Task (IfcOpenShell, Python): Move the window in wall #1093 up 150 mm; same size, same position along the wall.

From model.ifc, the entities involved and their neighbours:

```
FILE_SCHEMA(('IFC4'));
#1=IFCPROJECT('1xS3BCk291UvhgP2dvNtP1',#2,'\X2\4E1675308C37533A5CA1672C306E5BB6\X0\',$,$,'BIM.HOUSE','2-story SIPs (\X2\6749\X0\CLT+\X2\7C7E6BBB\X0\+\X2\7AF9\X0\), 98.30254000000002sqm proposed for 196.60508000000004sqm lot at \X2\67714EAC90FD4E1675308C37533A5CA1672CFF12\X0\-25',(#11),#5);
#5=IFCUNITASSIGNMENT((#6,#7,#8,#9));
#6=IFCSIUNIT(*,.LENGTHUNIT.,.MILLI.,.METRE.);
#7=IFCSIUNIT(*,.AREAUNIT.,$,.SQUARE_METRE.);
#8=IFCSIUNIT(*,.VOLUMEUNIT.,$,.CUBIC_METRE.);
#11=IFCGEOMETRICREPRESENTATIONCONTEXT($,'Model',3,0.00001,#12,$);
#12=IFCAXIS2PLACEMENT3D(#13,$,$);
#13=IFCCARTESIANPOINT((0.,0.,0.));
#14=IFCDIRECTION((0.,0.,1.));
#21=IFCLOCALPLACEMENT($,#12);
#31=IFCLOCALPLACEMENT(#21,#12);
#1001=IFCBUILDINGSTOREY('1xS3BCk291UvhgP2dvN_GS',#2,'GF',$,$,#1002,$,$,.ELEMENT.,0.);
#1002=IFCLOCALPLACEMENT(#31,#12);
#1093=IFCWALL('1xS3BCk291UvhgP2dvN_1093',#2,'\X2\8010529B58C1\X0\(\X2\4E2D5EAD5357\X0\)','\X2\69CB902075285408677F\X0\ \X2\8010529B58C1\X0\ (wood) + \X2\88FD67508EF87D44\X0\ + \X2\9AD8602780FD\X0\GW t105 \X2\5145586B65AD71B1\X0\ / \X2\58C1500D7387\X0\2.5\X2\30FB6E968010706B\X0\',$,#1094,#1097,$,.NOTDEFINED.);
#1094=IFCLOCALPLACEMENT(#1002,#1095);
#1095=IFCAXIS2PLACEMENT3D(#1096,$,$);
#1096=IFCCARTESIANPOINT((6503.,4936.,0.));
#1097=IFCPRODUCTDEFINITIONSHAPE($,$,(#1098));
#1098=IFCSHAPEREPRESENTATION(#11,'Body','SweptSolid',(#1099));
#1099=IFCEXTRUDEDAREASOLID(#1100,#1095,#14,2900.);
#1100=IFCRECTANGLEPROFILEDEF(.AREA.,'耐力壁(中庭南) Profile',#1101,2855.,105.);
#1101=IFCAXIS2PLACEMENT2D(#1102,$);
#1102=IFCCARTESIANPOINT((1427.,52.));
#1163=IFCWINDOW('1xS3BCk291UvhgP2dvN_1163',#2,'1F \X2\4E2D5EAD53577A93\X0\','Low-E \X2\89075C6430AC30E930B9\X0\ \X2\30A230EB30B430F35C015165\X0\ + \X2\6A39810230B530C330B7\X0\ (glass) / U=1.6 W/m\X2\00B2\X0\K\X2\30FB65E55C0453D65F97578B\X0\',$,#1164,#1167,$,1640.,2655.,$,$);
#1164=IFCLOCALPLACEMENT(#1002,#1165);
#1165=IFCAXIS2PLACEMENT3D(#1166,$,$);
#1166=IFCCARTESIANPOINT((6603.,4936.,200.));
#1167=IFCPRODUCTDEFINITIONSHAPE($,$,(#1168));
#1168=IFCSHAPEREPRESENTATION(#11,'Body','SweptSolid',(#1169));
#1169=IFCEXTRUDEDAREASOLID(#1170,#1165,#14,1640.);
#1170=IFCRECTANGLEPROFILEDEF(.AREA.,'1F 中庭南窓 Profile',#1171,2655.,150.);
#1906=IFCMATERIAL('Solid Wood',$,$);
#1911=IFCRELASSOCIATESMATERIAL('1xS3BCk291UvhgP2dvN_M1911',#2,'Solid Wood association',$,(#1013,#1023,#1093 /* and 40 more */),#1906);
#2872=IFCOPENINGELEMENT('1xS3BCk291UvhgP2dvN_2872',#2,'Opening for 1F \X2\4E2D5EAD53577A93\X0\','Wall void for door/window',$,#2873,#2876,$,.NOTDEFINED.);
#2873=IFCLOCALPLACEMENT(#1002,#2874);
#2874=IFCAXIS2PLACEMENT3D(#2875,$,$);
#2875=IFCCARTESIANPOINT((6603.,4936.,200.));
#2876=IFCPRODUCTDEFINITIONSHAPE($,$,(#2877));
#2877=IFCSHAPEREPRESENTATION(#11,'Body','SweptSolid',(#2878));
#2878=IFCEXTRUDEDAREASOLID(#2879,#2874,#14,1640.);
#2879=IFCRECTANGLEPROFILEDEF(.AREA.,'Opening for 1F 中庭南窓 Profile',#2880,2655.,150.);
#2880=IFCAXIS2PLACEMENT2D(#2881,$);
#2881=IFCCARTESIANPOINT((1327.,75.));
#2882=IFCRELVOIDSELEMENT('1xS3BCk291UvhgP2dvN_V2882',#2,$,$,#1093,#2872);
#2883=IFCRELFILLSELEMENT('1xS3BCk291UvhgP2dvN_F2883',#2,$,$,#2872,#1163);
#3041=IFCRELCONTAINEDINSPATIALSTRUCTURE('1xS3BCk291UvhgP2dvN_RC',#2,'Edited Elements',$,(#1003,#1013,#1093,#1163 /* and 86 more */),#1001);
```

```python
import numpy as np
import ifcopenshell
import ifcopenshell.api.geometry
import ifcopenshell.util.placement
import ifcopenshell.util.unit

model = ifcopenshell.open("model.ifc")
unit_scale = ifcopenshell.util.unit.calculate_unit_scale(model)

window = model.by_id(1163)
opening = window.FillsVoids[0].RelatingOpeningElement
dz = 150.0

shift = np.array([0.0, 0.0, dz])
# The window is not placed relative to its opening, so move both.
for product in (opening, window):
    matrix = ifcopenshell.util.placement.get_local_placement(product.ObjectPlacement)
    matrix[:3, 3] += shift
    ifcopenshell.api.geometry.edit_object_placement(model, product=product, matrix=matrix, is_si=False)

print(f"moved by {dz * unit_scale:+.3f} m")

model.write("model_rev.ifc")
```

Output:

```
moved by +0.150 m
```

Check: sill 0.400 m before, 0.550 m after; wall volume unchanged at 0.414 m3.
